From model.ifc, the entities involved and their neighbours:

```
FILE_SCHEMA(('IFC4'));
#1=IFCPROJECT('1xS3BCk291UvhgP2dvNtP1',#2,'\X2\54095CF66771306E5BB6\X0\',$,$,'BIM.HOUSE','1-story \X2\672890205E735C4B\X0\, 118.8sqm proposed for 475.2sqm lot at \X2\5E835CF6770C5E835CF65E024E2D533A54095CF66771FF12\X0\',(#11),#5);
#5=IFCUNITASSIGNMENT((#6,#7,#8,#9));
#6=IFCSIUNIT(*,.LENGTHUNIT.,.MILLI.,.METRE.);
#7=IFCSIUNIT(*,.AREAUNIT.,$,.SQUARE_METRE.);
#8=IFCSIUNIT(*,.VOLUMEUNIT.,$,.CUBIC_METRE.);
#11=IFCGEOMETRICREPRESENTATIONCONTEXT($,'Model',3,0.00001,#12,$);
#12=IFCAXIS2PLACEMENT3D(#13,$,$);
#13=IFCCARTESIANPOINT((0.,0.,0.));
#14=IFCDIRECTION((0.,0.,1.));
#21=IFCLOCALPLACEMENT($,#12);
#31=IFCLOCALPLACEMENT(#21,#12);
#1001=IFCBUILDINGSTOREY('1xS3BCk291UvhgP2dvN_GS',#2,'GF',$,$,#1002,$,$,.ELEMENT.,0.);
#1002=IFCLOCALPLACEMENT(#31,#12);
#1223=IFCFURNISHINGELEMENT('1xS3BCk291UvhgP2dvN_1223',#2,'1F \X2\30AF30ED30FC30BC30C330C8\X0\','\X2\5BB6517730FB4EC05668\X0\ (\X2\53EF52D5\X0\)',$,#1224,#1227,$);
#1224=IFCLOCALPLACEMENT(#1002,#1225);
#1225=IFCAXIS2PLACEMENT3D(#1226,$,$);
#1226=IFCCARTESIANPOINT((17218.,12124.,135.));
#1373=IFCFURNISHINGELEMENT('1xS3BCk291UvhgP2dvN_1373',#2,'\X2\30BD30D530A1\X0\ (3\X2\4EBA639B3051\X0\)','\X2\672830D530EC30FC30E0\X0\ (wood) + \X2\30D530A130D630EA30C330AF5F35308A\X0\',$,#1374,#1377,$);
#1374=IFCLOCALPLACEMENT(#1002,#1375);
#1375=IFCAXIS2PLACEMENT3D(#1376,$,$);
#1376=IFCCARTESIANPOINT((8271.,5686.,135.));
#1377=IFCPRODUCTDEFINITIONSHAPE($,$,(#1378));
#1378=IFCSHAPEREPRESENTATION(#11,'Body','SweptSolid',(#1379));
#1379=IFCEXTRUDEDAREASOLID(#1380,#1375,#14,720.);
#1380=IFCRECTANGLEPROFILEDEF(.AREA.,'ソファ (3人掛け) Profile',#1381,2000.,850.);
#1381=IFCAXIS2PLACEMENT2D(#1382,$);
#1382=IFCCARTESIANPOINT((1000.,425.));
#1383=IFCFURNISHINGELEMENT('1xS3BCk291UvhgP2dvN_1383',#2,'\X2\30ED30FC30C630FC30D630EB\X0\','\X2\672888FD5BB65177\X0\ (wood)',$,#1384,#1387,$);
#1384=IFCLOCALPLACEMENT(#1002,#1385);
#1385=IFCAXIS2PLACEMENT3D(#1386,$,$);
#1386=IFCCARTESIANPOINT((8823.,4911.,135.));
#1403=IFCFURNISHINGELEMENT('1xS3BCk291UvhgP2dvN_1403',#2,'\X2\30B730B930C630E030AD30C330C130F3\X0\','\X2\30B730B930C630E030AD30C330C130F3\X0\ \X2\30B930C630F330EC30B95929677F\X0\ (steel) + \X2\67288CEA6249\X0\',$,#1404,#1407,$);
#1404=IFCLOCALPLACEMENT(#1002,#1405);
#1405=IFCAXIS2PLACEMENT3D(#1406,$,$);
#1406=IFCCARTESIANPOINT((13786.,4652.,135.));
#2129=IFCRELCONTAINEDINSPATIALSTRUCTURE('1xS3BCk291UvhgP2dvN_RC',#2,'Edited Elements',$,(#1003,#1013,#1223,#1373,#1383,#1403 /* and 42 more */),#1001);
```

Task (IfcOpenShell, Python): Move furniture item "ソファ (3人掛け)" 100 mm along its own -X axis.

```python
import ifcopenshell
import ifcopenshell.api.geometry
import ifcopenshell.util.placement
import ifcopenshell.util.unit

model = ifcopenshell.open("model.ifc")
unit_scale = ifcopenshell.util.unit.calculate_unit_scale(model)

item = model.by_guid("1xS3BCk291UvhgP2dvN_1373")
matrix = ifcopenshell.util.placement.get_local_placement(item.ObjectPlacement)
matrix[:3, 3] -= matrix[:3, 0] * 0.1 / unit_scale
ifcopenshell.api.geometry.edit_object_placement(model, product=item, matrix=matrix, is_si=False)

print(ifcopenshell.util.placement.get_local_placement(item.ObjectPlacement).round(3) + 0.0)

model.write("model-out.ifc")
```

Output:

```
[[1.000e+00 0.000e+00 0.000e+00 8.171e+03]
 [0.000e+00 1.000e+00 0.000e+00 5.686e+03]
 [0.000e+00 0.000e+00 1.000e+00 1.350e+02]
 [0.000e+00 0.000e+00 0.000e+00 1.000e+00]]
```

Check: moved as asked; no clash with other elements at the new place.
